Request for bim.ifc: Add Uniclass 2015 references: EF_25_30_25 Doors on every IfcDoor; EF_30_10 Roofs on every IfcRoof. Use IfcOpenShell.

First a look at what the model holds.

```python
import ifcopenshell

model = ifcopenshell.open("bim.ifc")
print(model.schema)
print("classifications:", [c.Name for c in model.by_type("IfcClassification")])
for ifc_class in ("IfcDoor", "IfcRoof", "IfcStair", "IfcWall", "IfcWindow"):
    print(ifc_class, len(model.by_type(ifc_class)))
```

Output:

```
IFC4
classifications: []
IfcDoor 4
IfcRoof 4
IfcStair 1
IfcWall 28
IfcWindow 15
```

```python
import ifcopenshell
import ifcopenshell.api.classification

model = ifcopenshell.open("bim.ifc")

system = ifcopenshell.api.classification.add_classification(model, classification="Uniclass 2015")

codes = {
    "IfcDoor": ("EF_25_30_25", "Doors"),
    "IfcRoof": ("EF_30_10", "Roofs"),
}
for ifc_class, (code, name) in codes.items():
    products = model.by_type(ifc_class)
    ifcopenshell.api.classification.add_reference(
        model, products=products, classification=system, identification=code, name=name
    )
    print(code, len(products))

model.write("bim_v2.ifc")
```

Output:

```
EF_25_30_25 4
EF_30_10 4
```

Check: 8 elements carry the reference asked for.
